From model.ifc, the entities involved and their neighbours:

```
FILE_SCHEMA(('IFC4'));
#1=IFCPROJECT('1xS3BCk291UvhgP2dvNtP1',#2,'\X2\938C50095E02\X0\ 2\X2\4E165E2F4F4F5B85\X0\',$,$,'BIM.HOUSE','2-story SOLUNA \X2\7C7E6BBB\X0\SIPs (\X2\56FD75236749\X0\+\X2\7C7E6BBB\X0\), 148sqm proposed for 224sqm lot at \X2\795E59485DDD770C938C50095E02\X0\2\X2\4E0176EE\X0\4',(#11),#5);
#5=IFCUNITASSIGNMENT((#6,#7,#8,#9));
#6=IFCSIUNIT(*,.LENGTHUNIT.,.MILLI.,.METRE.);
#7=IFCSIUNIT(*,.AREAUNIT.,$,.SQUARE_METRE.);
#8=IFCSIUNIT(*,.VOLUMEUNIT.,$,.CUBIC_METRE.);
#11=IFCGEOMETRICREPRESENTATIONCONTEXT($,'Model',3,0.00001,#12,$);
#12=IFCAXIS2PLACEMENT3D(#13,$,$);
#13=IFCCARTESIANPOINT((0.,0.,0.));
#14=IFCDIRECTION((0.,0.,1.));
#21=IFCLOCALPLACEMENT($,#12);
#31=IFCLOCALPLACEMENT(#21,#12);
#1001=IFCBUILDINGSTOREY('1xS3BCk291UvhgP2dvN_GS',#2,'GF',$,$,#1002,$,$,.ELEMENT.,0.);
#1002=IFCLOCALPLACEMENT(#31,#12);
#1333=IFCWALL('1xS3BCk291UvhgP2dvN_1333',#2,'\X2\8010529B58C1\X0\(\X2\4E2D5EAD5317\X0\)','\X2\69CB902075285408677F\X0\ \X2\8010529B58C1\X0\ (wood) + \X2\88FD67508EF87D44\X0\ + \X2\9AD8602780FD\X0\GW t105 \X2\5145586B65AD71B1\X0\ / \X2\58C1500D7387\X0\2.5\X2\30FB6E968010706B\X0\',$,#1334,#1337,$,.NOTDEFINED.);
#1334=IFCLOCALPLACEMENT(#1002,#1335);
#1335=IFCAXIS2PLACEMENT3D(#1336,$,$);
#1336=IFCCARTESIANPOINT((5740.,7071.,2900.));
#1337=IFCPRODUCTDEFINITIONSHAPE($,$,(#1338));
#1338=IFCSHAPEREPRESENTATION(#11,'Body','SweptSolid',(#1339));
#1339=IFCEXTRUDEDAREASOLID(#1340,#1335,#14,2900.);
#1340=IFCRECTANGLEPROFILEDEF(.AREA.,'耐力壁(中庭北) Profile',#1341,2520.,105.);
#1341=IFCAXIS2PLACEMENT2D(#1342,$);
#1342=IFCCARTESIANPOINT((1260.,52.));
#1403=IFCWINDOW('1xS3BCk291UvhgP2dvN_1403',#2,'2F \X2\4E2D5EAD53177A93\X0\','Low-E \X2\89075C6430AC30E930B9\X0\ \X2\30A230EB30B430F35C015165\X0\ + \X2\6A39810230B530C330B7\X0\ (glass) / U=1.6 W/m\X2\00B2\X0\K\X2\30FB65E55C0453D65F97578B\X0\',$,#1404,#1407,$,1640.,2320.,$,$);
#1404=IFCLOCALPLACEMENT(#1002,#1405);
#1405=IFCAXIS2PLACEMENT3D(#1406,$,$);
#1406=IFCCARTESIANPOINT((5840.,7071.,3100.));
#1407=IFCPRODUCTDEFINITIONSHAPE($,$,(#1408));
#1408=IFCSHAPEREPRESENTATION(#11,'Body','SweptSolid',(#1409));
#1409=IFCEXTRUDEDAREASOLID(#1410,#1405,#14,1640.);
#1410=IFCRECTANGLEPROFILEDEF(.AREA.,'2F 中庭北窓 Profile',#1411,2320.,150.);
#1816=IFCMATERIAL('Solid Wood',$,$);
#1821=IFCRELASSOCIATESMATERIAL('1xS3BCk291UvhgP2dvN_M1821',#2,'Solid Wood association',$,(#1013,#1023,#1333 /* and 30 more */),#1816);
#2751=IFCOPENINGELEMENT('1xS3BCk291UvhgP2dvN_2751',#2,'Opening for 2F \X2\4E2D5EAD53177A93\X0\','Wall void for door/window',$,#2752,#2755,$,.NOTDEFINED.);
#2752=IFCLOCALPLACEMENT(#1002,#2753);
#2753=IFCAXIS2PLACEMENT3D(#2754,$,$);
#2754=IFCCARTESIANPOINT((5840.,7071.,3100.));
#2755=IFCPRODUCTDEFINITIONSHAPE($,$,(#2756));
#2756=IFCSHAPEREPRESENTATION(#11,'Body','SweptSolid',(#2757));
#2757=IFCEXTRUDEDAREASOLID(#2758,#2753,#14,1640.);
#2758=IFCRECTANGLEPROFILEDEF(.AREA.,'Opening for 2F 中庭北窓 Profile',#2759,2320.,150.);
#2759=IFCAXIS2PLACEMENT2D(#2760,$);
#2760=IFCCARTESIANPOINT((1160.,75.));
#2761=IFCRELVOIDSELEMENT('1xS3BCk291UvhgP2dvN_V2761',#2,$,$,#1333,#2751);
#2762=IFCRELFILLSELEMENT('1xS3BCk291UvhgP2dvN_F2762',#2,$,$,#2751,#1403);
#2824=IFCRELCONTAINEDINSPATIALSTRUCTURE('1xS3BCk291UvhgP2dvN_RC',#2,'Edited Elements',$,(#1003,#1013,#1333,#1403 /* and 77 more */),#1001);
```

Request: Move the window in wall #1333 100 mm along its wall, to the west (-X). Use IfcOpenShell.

```python
import ifcopenshell
import ifcopenshell.api.geometry
import ifcopenshell.util.placement
import ifcopenshell.util.unit

model = ifcopenshell.open("model.ifc")
unit_scale = ifcopenshell.util.unit.calculate_unit_scale(model)

window = model.by_id(1403)
opening = window.FillsVoids[0].RelatingOpeningElement
wall = opening.VoidsElements[0].RelatingBuildingElement

wall_matrix = ifcopenshell.util.placement.get_local_placement(wall.ObjectPlacement)
shift = wall_matrix[:3, 0] * -0.1 / unit_scale
before = ifcopenshell.util.placement.get_local_placement(window.ObjectPlacement)[:3, 3].copy()

# The window is not placed relative to its opening, so move both.
for product in (opening, window):
    matrix = ifcopenshell.util.placement.get_local_placement(product.ObjectPlacement)
    matrix[:3, 3] += shift
    ifcopenshell.api.geometry.edit_object_placement(model, product=product, matrix=matrix, is_si=False)

after = ifcopenshell.util.placement.get_local_placement(window.ObjectPlacement)[:3, 3]
print("window moved by", (after - before).round(3) + 0.0)

model.write("model_edited.ifc")
```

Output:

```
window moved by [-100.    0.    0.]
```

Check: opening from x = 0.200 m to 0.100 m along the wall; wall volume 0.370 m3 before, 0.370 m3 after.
